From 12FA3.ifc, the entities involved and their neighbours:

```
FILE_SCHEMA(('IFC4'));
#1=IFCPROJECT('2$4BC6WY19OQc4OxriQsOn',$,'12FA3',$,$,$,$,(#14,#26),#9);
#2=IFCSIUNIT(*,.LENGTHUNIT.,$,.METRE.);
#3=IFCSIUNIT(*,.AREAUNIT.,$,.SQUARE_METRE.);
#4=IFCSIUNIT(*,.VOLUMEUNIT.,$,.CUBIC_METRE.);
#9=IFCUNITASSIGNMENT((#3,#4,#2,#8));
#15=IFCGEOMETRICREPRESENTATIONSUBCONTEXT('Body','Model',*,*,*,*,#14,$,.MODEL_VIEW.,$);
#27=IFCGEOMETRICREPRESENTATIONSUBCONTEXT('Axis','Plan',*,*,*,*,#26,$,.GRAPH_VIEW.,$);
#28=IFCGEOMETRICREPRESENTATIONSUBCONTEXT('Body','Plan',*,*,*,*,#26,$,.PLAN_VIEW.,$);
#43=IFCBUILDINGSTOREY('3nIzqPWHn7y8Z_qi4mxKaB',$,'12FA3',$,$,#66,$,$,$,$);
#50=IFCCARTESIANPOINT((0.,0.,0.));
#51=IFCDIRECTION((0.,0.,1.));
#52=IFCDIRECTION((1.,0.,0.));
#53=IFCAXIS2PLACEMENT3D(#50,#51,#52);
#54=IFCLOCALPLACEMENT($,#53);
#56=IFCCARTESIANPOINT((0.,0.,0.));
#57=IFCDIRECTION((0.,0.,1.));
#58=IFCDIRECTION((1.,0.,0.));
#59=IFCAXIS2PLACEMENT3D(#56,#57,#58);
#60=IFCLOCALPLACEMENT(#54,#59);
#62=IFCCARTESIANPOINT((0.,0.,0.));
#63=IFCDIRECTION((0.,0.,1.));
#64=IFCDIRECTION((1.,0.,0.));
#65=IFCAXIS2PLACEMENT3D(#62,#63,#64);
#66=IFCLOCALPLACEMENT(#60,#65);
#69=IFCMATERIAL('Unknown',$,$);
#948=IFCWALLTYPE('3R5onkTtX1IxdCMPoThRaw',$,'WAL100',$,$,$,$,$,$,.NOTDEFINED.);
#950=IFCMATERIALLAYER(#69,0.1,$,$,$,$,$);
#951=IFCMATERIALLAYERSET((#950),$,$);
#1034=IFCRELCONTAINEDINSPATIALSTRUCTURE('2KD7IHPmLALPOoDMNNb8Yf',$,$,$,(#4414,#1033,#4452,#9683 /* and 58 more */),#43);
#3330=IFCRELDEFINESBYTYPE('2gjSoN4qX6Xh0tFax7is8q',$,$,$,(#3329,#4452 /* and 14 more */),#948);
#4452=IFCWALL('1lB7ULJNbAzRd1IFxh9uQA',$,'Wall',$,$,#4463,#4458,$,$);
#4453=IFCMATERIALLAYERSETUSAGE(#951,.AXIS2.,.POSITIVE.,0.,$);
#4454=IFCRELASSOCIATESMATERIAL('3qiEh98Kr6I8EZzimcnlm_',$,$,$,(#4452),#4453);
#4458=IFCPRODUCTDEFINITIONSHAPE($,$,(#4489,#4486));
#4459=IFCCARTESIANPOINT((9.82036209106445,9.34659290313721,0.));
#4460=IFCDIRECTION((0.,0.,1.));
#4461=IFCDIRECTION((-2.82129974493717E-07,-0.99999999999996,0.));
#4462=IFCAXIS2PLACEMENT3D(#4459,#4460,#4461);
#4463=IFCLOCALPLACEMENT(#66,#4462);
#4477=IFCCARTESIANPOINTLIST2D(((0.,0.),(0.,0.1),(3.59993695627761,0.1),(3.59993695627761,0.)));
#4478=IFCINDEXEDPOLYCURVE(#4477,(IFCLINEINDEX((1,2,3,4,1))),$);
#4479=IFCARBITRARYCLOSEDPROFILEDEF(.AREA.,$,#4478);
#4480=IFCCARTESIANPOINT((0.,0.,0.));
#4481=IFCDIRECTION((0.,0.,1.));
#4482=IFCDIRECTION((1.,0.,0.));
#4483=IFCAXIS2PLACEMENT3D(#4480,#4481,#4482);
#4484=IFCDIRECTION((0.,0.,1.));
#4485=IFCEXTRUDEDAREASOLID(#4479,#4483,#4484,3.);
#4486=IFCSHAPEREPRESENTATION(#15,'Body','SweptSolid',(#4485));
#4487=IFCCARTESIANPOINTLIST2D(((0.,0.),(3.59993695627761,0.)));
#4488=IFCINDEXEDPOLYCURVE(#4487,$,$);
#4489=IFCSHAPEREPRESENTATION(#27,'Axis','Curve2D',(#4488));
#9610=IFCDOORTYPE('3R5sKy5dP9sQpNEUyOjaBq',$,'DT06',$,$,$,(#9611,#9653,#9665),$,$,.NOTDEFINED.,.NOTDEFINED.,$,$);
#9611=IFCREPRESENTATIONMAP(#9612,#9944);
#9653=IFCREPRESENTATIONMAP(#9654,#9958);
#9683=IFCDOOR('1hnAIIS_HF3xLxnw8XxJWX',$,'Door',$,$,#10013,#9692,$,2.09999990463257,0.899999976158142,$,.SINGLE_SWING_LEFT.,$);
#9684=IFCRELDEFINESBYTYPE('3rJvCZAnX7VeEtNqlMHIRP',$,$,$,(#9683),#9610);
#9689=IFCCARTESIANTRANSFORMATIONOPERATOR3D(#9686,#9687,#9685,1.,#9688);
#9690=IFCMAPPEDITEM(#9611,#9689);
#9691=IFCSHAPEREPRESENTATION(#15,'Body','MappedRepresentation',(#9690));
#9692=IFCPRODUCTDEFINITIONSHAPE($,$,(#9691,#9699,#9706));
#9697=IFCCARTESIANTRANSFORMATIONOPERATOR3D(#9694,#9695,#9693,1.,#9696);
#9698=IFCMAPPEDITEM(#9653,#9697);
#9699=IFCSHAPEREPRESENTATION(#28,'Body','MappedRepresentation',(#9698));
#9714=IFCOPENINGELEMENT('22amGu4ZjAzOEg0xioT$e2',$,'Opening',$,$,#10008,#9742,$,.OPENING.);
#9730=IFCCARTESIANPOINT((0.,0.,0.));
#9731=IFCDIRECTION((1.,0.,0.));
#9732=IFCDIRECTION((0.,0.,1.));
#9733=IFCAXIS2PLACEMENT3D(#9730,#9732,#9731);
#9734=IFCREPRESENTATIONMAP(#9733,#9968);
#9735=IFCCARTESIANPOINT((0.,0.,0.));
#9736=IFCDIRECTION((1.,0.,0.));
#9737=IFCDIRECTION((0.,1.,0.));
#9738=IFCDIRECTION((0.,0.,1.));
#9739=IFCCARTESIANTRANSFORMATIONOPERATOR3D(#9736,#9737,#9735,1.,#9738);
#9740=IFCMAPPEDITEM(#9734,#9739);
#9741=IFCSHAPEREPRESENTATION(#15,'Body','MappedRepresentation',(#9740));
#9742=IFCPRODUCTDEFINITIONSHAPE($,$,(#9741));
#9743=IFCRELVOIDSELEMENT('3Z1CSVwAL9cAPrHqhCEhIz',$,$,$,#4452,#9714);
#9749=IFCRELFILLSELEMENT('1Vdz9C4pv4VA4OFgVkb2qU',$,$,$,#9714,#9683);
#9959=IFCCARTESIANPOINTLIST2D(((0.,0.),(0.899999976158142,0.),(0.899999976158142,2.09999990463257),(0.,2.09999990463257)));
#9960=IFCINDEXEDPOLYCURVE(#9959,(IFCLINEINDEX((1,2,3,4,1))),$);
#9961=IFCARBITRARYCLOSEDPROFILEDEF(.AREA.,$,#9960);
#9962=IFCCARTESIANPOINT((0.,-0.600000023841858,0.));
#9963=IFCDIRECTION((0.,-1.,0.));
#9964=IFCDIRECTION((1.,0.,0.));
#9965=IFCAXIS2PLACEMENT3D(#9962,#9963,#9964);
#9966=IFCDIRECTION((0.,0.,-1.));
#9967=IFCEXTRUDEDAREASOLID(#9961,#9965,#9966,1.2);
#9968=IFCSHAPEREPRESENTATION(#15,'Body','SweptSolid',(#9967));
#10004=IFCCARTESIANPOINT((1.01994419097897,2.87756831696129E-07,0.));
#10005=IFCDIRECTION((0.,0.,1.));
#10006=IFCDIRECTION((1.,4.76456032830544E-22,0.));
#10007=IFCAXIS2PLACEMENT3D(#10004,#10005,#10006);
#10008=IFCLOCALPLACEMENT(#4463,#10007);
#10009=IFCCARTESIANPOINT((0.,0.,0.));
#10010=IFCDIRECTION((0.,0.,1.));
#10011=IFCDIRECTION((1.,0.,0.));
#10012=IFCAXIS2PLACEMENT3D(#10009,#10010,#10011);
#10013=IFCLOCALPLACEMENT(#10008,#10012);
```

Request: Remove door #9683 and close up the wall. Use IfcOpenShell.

```python
import ifcopenshell
import ifcopenshell.api.feature
import ifcopenshell.api.root
import ifcopenshell.geom
import ifcopenshell.util.shape

model = ifcopenshell.open("12FA3.ifc")
settings = ifcopenshell.geom.settings()


def volume(element):
    """Net volume in cubic metres, openings subtracted."""
    shape = ifcopenshell.geom.create_shape(settings, element)
    return ifcopenshell.util.shape.get_volume(shape.geometry)


door = model.by_guid("1hnAIIS_HF3xLxnw8XxJWX")
opening = door.FillsVoids[0].RelatingOpeningElement
wall = opening.VoidsElements[0].RelatingBuildingElement
before = volume(wall)

ifcopenshell.api.root.remove_product(model, product=door)
ifcopenshell.api.feature.remove_feature(model, feature=opening)

after = volume(wall)

print(f"wall volume {before:.3f} -> {after:.3f} m3")

model.write("12FA3_edited.ifc")
```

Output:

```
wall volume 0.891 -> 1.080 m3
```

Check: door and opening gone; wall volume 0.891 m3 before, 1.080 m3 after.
